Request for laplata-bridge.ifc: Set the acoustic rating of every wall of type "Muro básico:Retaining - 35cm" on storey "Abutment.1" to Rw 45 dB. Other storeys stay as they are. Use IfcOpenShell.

First a look at what the model holds.

```python
import ifcopenshell
import ifcopenshell.util.element

model = ifcopenshell.open("laplata-bridge.ifc")
print(model.schema)
storey = next(s for s in model.by_type("IfcBuildingStorey") if s.Name == "Abutment.1")
walls = [e for e in ifcopenshell.util.element.get_decomposition(storey) if e.is_a("IfcWall")]
seen = {}
for e in walls:
    element_type = ifcopenshell.util.element.get_type(e)
    key = (element_type.Name if element_type != e and element_type else None, ifcopenshell.util.element.get_pset(e, "Pset_WallCommon", "AcousticRating"))
    seen[key] = seen.get(key, 0) + 1
for (name, value), count in sorted(seen.items(), key=str):
    print(count, "x", name, "|", value)
```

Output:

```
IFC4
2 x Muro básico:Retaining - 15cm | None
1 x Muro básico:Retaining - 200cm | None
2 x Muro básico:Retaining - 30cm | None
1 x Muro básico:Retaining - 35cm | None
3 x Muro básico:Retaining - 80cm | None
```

```python
import ifcopenshell
import ifcopenshell.api.pset
import ifcopenshell.util.element

model = ifcopenshell.open("laplata-bridge.ifc")

storey = next(s for s in model.by_type("IfcBuildingStorey") if s.Name == "Abutment.1")
walls = [e for e in ifcopenshell.util.element.get_decomposition(storey) if e.is_a("IfcWall")]

count = 0
for e in walls:
    element_type = ifcopenshell.util.element.get_type(e)
    if element_type in (None, e) or element_type.Name != "Muro básico:Retaining - 35cm":
        continue
    # add_pset returns the element's existing set when there is one.
    pset = ifcopenshell.api.pset.add_pset(model, product=e, name="Pset_WallCommon")
    ifcopenshell.api.pset.edit_pset(model, pset=pset, properties={"AcousticRating": "Rw 45 dB"})
    count += 1

print(count, "walls updated")

model.write("laplata-bridge_updated.ifc")
```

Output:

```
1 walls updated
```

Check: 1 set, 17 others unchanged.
